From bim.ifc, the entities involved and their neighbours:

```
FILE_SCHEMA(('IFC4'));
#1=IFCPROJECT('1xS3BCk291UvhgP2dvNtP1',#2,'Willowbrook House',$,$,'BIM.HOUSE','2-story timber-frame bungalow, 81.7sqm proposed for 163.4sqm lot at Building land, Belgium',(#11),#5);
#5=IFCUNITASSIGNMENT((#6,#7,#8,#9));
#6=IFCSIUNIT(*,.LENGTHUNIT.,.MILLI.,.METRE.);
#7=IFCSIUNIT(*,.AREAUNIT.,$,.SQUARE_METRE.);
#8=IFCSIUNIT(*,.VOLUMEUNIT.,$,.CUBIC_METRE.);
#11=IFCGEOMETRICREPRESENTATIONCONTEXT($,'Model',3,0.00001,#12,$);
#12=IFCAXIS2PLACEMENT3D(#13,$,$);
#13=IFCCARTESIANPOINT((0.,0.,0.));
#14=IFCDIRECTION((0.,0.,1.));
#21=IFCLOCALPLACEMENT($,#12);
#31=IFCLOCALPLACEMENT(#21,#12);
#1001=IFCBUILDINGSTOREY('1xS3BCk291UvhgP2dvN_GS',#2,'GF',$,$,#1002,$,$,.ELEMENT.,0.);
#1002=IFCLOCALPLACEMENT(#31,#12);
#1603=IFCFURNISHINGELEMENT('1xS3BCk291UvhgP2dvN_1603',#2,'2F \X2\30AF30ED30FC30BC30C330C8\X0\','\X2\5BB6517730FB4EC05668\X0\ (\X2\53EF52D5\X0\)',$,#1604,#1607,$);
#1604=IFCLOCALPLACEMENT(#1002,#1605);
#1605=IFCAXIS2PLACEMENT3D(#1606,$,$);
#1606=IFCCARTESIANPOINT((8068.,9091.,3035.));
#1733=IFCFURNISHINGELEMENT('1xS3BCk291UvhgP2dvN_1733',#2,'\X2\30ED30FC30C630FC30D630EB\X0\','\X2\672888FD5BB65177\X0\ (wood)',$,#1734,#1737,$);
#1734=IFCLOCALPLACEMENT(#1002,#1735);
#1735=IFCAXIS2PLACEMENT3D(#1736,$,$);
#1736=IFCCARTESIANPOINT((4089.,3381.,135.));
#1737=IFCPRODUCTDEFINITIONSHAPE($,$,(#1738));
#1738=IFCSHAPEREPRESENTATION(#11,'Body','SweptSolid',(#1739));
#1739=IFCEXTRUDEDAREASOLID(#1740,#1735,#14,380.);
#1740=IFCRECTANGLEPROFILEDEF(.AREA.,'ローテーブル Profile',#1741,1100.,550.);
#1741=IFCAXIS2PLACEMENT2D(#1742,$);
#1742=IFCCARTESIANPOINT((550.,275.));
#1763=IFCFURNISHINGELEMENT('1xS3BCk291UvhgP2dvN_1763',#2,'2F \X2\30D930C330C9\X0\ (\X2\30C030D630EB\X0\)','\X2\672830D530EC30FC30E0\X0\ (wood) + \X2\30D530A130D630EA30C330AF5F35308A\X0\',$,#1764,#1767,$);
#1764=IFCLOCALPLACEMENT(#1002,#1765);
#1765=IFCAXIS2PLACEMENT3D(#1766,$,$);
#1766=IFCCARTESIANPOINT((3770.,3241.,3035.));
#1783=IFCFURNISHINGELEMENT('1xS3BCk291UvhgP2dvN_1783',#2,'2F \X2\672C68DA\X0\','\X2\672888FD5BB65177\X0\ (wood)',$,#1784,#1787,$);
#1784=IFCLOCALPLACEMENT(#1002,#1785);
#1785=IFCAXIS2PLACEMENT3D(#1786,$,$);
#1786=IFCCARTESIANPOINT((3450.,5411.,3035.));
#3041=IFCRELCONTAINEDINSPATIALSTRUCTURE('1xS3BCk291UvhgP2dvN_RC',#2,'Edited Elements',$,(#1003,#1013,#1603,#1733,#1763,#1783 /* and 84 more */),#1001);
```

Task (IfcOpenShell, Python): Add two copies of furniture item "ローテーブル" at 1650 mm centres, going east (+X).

```python
import numpy as np
import ifcopenshell
import ifcopenshell.api.geometry
import ifcopenshell.api.root
import ifcopenshell.util.element
import ifcopenshell.util.placement
import ifcopenshell.util.unit

model = ifcopenshell.open("bim.ifc")
unit_scale = ifcopenshell.util.unit.calculate_unit_scale(model)


def reuse_history(source, copy):
    """copy_class also copies each property set's owner history, people and application; keep the originals."""
    for rel in copy.IsDefinedBy:
        if rel.is_a("IfcRelDefinesByProperties") and (history := rel.RelatingPropertyDefinition.OwnerHistory):
            rel.RelatingPropertyDefinition.OwnerHistory = source.OwnerHistory
            ifcopenshell.util.element.remove_deep2(model, history)


source = model.by_guid("1xS3BCk291UvhgP2dvN_1733")
base = ifcopenshell.util.placement.get_local_placement(source.ObjectPlacement)
step = np.array([1.0, 0.0, 0.0]) * 1.65 / unit_scale

for i in range(1, 3):
    copy = ifcopenshell.api.root.copy_class(model, product=source)
    copy.Representation = ifcopenshell.util.element.copy_deep(
        model, source.Representation, exclude=["IfcGeometricRepresentationContext", "IfcRepresentationMap"]
    )
    reuse_history(source, copy)
    matrix = base.copy()
    matrix[:3, 3] += i * step
    print("added at", matrix[:3, 3].round(3) + 0.0)
    ifcopenshell.api.geometry.edit_object_placement(model, product=copy, matrix=matrix, is_si=False)

model.write("bim_rev.ifc")
```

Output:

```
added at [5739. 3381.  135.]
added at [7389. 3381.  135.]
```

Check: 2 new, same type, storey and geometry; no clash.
